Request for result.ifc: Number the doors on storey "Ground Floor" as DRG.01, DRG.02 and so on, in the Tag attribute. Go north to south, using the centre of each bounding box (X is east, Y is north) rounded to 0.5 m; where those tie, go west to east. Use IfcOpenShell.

First a look at what the model holds.

```python
import ifcopenshell
import ifcopenshell.util.element
import ifcopenshell.util.placement

model = ifcopenshell.open("result.ifc")
print(model.schema)
storey = next(s for s in model.by_type("IfcBuildingStorey") if s.Name == "Ground Floor")
doors = [e for e in ifcopenshell.util.element.get_decomposition(storey) if e.is_a("IfcDoor")]
for e in sorted(doors, key=lambda e: e.id()):
    origin = ifcopenshell.util.placement.get_local_placement(e.ObjectPlacement)[:3, 3]
    print(e.id(), e.Tag, e.Name, origin.round(2) + 0.0, sep=" | ")
```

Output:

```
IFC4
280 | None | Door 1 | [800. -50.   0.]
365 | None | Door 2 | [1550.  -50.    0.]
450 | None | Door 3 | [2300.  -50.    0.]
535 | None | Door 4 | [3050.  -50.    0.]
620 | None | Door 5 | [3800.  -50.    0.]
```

```python
import ifcopenshell
import ifcopenshell.geom
import ifcopenshell.util.element
import ifcopenshell.util.shape

model = ifcopenshell.open("result.ifc")
settings = ifcopenshell.geom.settings()
settings.set("use-world-coords", True)


def centre(element):
    shape = ifcopenshell.geom.create_shape(settings, element)
    return ifcopenshell.util.shape.get_bbox_centroid(shape.geometry)


storey = next(s for s in model.by_type("IfcBuildingStorey") if s.Name == "Ground Floor")
doors = [e for e in ifcopenshell.util.element.get_decomposition(storey) if e.is_a("IfcDoor")]

# Insertion points can sit at a corner or the storey origin, so sort by the geometry (in metres).
centres = {e: centre(e) for e in doors}
doors.sort(key=lambda e: (-round(centres[e][1] / 0.5), centres[e][0]))

for i, e in enumerate(doors, start=1):
    number = f"DRG.{i:02d}"
    e.Tag = number
    print(e.id(), number)

model.write("result_edited.ifc")
```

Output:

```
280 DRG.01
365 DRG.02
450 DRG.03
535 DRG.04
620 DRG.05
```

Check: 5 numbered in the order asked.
